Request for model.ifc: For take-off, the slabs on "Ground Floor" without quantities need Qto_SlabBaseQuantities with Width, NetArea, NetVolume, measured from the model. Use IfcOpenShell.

First a look at what the model holds.

```python
import ifcopenshell
import ifcopenshell.util.element
import ifcopenshell.util.unit

model = ifcopenshell.open("model.ifc")
print(model.schema)
for unit_type in ("LENGTHUNIT", "AREAUNIT", "VOLUMEUNIT"):
    print(unit_type, ifcopenshell.util.unit.calculate_unit_scale(model, unit_type))
storey = next(s for s in model.by_type("IfcBuildingStorey") if s.Name == "Ground Floor")
slabs = [e for e in ifcopenshell.util.element.get_decomposition(storey) if e.is_a("IfcSlab")]
for e in sorted(slabs, key=lambda e: e.id()):
    print(e.id(), e.is_a(), e.Name, list(ifcopenshell.util.element.get_psets(e, qtos_only=True)), sep=" | ")
```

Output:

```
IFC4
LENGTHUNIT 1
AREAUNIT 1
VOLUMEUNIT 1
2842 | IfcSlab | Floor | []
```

```python
import ifcopenshell
import ifcopenshell.api.pset
import ifcopenshell.geom
import ifcopenshell.util.element
import ifcopenshell.util.shape
import ifcopenshell.util.unit

model = ifcopenshell.open("model.ifc")
unit_scale = ifcopenshell.util.unit.calculate_unit_scale(model)
area_scale = ifcopenshell.util.unit.calculate_unit_scale(model, "AREAUNIT")
volume_scale = ifcopenshell.util.unit.calculate_unit_scale(model, "VOLUMEUNIT")
settings = ifcopenshell.geom.settings()

storey = next(s for s in model.by_type("IfcBuildingStorey") if s.Name == "Ground Floor")
slabs = [e for e in ifcopenshell.util.element.get_decomposition(storey) if e.is_a("IfcSlab")]

for e in sorted(slabs, key=lambda e: e.id()):
    if ifcopenshell.util.element.get_psets(e, qtos_only=True, should_inherit=False):
        continue
    # Geometry comes back in metres, in the element's own axes.
    shape = ifcopenshell.geom.create_shape(settings, e)
    values = {
        "Width": ifcopenshell.util.shape.get_z(shape.geometry) / unit_scale,
        "NetArea": ifcopenshell.util.shape.get_footprint_area(shape.geometry) / area_scale,
        "NetVolume": ifcopenshell.util.shape.get_volume(shape.geometry) / volume_scale,
    }
    qto = ifcopenshell.api.pset.add_qto(model, product=e, name="Qto_SlabBaseQuantities")
    ifcopenshell.api.pset.edit_qto(model, qto=qto, properties=values)
    print(e.id(), {k: round(v, 3) for k, v in values.items()})

model.write("model_edited.ifc")
```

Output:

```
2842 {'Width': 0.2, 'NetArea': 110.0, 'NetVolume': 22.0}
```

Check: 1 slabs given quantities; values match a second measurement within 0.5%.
